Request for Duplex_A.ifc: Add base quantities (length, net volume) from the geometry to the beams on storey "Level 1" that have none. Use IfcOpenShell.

First a look at what the model holds.

```python
import ifcopenshell
import ifcopenshell.util.element
import ifcopenshell.util.unit

model = ifcopenshell.open("Duplex_A.ifc")
print(model.schema)
for unit_type in ("LENGTHUNIT", "AREAUNIT", "VOLUMEUNIT"):
    print(unit_type, ifcopenshell.util.unit.calculate_unit_scale(model, unit_type))
storey = next(s for s in model.by_type("IfcBuildingStorey") if s.Name == "Level 1")
beams = [e for e in ifcopenshell.util.element.get_decomposition(storey) if e.is_a("IfcBeam")]
for e in sorted(beams, key=lambda e: e.id()):
    print(e.id(), e.is_a(), e.Name, list(ifcopenshell.util.element.get_psets(e, qtos_only=True)), sep=" | ")
```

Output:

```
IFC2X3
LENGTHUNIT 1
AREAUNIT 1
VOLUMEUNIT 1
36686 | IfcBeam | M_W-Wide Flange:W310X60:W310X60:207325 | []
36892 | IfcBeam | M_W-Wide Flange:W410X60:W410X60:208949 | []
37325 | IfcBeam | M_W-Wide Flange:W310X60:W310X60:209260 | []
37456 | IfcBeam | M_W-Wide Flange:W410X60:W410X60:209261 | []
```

```python
import ifcopenshell
import ifcopenshell.api.pset
import ifcopenshell.geom
import ifcopenshell.util.element
import ifcopenshell.util.shape
import ifcopenshell.util.unit

model = ifcopenshell.open("Duplex_A.ifc")
unit_scale = ifcopenshell.util.unit.calculate_unit_scale(model)
volume_scale = ifcopenshell.util.unit.calculate_unit_scale(model, "VOLUMEUNIT")
settings = ifcopenshell.geom.settings()

storey = next(s for s in model.by_type("IfcBuildingStorey") if s.Name == "Level 1")
beams = [e for e in ifcopenshell.util.element.get_decomposition(storey) if e.is_a("IfcBeam")]

for e in sorted(beams, key=lambda e: e.id()):
    if ifcopenshell.util.element.get_psets(e, qtos_only=True, should_inherit=False):
        continue
    # Geometry comes back in metres, in the element's own axes.
    shape = ifcopenshell.geom.create_shape(settings, e)
    values = {
        "Length": ifcopenshell.util.shape.get_max_xyz(shape.geometry) / unit_scale,
        "NetVolume": ifcopenshell.util.shape.get_volume(shape.geometry) / volume_scale,
    }
    qto = ifcopenshell.api.pset.add_qto(model, product=e, name="BaseQuantities")
    ifcopenshell.api.pset.edit_qto(model, qto=qto, properties=values)
    print(e.id(), {k: round(v, 3) for k, v in values.items()})

model.write("Duplex_A-out.ifc")
```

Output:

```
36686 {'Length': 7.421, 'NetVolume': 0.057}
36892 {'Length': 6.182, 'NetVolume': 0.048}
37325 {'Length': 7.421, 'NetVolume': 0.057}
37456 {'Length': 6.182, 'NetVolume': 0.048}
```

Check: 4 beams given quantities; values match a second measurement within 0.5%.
